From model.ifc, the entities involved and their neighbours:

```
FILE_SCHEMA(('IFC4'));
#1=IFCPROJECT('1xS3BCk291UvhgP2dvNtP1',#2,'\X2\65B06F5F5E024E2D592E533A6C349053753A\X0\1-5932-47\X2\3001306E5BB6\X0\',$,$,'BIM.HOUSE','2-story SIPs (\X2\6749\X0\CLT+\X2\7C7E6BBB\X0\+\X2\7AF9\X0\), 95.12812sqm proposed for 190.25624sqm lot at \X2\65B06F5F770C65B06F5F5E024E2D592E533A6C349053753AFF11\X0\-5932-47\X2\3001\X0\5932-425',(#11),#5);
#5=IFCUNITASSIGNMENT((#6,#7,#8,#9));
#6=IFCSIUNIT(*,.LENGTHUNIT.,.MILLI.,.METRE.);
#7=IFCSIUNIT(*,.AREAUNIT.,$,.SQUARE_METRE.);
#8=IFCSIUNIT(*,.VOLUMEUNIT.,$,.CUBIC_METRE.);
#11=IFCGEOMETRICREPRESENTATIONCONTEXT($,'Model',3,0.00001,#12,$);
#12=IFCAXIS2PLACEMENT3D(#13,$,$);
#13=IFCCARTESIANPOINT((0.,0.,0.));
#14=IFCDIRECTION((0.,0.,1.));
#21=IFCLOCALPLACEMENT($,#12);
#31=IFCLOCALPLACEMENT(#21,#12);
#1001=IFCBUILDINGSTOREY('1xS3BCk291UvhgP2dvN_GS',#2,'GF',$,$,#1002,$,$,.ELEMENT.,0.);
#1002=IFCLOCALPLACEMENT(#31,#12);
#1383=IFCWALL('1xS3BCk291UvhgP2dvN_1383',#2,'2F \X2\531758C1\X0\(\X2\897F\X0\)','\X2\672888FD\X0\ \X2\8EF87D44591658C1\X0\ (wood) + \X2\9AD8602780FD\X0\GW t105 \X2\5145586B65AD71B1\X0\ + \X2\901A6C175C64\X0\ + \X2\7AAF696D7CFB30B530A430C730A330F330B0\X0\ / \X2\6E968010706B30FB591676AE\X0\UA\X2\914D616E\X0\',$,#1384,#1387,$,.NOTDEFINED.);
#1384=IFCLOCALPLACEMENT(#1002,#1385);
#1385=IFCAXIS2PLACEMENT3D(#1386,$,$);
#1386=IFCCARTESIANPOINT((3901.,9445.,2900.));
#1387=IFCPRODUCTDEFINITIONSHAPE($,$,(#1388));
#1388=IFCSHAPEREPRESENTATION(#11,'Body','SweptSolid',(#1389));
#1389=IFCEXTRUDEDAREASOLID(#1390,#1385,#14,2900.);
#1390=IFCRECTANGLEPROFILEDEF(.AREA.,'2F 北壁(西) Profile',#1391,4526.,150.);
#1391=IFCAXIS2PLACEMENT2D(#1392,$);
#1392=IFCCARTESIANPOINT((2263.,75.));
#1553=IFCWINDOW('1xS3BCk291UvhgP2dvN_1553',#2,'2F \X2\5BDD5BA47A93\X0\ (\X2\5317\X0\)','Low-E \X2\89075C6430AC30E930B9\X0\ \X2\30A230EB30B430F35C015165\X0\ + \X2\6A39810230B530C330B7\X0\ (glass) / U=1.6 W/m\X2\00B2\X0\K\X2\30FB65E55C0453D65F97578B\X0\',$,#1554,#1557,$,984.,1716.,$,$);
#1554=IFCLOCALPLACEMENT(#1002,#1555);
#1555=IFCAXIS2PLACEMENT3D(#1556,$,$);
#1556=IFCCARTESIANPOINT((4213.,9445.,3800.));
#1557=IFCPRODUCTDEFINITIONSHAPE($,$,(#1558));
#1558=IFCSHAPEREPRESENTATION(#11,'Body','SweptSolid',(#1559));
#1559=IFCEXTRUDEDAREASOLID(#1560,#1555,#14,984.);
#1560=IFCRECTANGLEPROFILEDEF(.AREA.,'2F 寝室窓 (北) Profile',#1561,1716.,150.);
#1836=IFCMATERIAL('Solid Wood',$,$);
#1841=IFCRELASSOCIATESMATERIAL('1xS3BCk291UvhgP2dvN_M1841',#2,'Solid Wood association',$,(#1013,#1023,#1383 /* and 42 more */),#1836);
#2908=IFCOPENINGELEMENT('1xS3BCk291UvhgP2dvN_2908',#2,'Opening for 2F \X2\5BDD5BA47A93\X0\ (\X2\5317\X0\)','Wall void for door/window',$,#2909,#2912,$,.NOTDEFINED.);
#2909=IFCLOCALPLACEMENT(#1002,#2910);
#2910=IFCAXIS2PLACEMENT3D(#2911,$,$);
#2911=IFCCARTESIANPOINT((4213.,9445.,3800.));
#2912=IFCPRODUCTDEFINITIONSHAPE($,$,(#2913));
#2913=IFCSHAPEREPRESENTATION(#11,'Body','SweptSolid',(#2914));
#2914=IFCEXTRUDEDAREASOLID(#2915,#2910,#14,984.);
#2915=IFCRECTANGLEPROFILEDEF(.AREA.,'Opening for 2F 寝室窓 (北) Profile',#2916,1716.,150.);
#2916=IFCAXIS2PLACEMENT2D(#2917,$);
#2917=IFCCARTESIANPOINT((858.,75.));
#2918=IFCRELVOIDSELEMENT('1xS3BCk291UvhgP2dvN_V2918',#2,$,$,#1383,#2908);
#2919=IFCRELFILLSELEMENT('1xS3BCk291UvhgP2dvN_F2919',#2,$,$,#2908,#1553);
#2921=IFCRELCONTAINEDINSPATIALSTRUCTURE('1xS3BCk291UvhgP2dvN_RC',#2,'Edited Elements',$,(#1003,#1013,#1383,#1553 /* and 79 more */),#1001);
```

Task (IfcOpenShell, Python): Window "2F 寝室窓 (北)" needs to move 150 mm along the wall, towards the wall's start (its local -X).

```python
import ifcopenshell
import ifcopenshell.api.geometry
import ifcopenshell.util.placement

model = ifcopenshell.open("model.ifc")

window = model.by_id(1553)
opening = window.FillsVoids[0].RelatingOpeningElement
wall = opening.VoidsElements[0].RelatingBuildingElement

wall_matrix = ifcopenshell.util.placement.get_local_placement(wall.ObjectPlacement)
shift = wall_matrix[:3, 0] * -150.0
before = ifcopenshell.util.placement.get_local_placement(window.ObjectPlacement)[:3, 3].copy()

# The window is not placed relative to its opening, so move both.
for product in (opening, window):
    matrix = ifcopenshell.util.placement.get_local_placement(product.ObjectPlacement)
    matrix[:3, 3] += shift
    ifcopenshell.api.geometry.edit_object_placement(model, product=product, matrix=matrix, is_si=False)

after = ifcopenshell.util.placement.get_local_placement(window.ObjectPlacement)[:3, 3]
print("window moved by", (after - before).round(3) + 0.0)

model.write("model_updated.ifc")
```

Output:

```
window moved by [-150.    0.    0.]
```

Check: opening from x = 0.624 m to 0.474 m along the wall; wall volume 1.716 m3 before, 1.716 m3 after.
